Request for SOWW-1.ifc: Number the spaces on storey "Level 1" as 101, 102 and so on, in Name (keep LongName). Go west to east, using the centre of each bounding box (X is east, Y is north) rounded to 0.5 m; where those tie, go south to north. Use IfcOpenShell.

First a look at what the model holds.

```python
import ifcopenshell
import ifcopenshell.util.element
import ifcopenshell.util.placement

model = ifcopenshell.open("SOWW-1.ifc")
print(model.schema)
storey = next(s for s in model.by_type("IfcBuildingStorey") if s.Name == "Level 1")
spaces = [e for e in ifcopenshell.util.element.get_decomposition(storey) if e.is_a("IfcSpace")]
for e in sorted(spaces, key=lambda e: e.id()):
    origin = ifcopenshell.util.placement.get_local_placement(e.ObjectPlacement)[:3, 3]
    print(e.id(), e.Name, e.LongName, origin.round(2) + 0.0, sep=" | ")
```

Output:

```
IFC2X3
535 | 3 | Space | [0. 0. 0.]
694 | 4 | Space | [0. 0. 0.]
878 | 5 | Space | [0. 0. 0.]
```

```python
import ifcopenshell
import ifcopenshell.geom
import ifcopenshell.util.element
import ifcopenshell.util.shape

model = ifcopenshell.open("SOWW-1.ifc")
settings = ifcopenshell.geom.settings()
settings.set("use-world-coords", True)


def centre(element):
    shape = ifcopenshell.geom.create_shape(settings, element)
    return ifcopenshell.util.shape.get_bbox_centroid(shape.geometry)


storey = next(s for s in model.by_type("IfcBuildingStorey") if s.Name == "Level 1")
spaces = [e for e in ifcopenshell.util.element.get_decomposition(storey) if e.is_a("IfcSpace")]

# Insertion points can sit at a corner or the storey origin, so sort by the geometry (in metres).
centres = {e: centre(e) for e in spaces}
spaces.sort(key=lambda e: (round(centres[e][0] / 0.5), centres[e][1]))

for i, e in enumerate(spaces, start=1):
    number = f"1{i:02d}"
    e.Name = number
    print(e.id(), number)

model.write("SOWW-1_rev.ifc")
```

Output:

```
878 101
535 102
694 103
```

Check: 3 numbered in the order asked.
